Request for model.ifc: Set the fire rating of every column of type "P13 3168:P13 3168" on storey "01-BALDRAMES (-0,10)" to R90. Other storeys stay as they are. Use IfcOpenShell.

First a look at what the model holds.

```python
import ifcopenshell
import ifcopenshell.util.element

model = ifcopenshell.open("model.ifc")
print(model.schema)
storey = next(s for s in model.by_type("IfcBuildingStorey") if s.Name == "01-BALDRAMES (-0,10)")
columns = [e for e in ifcopenshell.util.element.get_decomposition(storey) if e.is_a("IfcColumn")]
seen = {}
for e in columns:
    element_type = ifcopenshell.util.element.get_type(e)
    key = (element_type.Name if element_type != e and element_type else None, ifcopenshell.util.element.get_pset(e, "Pset_ColumnCommon", "FireRating"))
    seen[key] = seen.get(key, 0) + 1
for (name, value), count in sorted(seen.items(), key=str):
    print(count, "x", name, "|", value)
```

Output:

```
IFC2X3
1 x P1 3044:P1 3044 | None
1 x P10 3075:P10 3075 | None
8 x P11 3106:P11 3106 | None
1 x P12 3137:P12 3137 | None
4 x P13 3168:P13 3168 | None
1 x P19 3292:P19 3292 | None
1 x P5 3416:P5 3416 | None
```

```python
import ifcopenshell
import ifcopenshell.api.pset
import ifcopenshell.util.element

model = ifcopenshell.open("model.ifc")

storey = next(s for s in model.by_type("IfcBuildingStorey") if s.Name == "01-BALDRAMES (-0,10)")
columns = [e for e in ifcopenshell.util.element.get_decomposition(storey) if e.is_a("IfcColumn")]

count = 0
for e in columns:
    element_type = ifcopenshell.util.element.get_type(e)
    if element_type in (None, e) or element_type.Name != "P13 3168:P13 3168":
        continue
    # add_pset returns the element's existing set when there is one.
    pset = ifcopenshell.api.pset.add_pset(model, product=e, name="Pset_ColumnCommon")
    ifcopenshell.api.pset.edit_pset(model, pset=pset, properties={"FireRating": "R90"})
    count += 1

print(count, "columns updated")

model.write("model_v2.ifc")
```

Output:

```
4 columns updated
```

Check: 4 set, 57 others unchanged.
